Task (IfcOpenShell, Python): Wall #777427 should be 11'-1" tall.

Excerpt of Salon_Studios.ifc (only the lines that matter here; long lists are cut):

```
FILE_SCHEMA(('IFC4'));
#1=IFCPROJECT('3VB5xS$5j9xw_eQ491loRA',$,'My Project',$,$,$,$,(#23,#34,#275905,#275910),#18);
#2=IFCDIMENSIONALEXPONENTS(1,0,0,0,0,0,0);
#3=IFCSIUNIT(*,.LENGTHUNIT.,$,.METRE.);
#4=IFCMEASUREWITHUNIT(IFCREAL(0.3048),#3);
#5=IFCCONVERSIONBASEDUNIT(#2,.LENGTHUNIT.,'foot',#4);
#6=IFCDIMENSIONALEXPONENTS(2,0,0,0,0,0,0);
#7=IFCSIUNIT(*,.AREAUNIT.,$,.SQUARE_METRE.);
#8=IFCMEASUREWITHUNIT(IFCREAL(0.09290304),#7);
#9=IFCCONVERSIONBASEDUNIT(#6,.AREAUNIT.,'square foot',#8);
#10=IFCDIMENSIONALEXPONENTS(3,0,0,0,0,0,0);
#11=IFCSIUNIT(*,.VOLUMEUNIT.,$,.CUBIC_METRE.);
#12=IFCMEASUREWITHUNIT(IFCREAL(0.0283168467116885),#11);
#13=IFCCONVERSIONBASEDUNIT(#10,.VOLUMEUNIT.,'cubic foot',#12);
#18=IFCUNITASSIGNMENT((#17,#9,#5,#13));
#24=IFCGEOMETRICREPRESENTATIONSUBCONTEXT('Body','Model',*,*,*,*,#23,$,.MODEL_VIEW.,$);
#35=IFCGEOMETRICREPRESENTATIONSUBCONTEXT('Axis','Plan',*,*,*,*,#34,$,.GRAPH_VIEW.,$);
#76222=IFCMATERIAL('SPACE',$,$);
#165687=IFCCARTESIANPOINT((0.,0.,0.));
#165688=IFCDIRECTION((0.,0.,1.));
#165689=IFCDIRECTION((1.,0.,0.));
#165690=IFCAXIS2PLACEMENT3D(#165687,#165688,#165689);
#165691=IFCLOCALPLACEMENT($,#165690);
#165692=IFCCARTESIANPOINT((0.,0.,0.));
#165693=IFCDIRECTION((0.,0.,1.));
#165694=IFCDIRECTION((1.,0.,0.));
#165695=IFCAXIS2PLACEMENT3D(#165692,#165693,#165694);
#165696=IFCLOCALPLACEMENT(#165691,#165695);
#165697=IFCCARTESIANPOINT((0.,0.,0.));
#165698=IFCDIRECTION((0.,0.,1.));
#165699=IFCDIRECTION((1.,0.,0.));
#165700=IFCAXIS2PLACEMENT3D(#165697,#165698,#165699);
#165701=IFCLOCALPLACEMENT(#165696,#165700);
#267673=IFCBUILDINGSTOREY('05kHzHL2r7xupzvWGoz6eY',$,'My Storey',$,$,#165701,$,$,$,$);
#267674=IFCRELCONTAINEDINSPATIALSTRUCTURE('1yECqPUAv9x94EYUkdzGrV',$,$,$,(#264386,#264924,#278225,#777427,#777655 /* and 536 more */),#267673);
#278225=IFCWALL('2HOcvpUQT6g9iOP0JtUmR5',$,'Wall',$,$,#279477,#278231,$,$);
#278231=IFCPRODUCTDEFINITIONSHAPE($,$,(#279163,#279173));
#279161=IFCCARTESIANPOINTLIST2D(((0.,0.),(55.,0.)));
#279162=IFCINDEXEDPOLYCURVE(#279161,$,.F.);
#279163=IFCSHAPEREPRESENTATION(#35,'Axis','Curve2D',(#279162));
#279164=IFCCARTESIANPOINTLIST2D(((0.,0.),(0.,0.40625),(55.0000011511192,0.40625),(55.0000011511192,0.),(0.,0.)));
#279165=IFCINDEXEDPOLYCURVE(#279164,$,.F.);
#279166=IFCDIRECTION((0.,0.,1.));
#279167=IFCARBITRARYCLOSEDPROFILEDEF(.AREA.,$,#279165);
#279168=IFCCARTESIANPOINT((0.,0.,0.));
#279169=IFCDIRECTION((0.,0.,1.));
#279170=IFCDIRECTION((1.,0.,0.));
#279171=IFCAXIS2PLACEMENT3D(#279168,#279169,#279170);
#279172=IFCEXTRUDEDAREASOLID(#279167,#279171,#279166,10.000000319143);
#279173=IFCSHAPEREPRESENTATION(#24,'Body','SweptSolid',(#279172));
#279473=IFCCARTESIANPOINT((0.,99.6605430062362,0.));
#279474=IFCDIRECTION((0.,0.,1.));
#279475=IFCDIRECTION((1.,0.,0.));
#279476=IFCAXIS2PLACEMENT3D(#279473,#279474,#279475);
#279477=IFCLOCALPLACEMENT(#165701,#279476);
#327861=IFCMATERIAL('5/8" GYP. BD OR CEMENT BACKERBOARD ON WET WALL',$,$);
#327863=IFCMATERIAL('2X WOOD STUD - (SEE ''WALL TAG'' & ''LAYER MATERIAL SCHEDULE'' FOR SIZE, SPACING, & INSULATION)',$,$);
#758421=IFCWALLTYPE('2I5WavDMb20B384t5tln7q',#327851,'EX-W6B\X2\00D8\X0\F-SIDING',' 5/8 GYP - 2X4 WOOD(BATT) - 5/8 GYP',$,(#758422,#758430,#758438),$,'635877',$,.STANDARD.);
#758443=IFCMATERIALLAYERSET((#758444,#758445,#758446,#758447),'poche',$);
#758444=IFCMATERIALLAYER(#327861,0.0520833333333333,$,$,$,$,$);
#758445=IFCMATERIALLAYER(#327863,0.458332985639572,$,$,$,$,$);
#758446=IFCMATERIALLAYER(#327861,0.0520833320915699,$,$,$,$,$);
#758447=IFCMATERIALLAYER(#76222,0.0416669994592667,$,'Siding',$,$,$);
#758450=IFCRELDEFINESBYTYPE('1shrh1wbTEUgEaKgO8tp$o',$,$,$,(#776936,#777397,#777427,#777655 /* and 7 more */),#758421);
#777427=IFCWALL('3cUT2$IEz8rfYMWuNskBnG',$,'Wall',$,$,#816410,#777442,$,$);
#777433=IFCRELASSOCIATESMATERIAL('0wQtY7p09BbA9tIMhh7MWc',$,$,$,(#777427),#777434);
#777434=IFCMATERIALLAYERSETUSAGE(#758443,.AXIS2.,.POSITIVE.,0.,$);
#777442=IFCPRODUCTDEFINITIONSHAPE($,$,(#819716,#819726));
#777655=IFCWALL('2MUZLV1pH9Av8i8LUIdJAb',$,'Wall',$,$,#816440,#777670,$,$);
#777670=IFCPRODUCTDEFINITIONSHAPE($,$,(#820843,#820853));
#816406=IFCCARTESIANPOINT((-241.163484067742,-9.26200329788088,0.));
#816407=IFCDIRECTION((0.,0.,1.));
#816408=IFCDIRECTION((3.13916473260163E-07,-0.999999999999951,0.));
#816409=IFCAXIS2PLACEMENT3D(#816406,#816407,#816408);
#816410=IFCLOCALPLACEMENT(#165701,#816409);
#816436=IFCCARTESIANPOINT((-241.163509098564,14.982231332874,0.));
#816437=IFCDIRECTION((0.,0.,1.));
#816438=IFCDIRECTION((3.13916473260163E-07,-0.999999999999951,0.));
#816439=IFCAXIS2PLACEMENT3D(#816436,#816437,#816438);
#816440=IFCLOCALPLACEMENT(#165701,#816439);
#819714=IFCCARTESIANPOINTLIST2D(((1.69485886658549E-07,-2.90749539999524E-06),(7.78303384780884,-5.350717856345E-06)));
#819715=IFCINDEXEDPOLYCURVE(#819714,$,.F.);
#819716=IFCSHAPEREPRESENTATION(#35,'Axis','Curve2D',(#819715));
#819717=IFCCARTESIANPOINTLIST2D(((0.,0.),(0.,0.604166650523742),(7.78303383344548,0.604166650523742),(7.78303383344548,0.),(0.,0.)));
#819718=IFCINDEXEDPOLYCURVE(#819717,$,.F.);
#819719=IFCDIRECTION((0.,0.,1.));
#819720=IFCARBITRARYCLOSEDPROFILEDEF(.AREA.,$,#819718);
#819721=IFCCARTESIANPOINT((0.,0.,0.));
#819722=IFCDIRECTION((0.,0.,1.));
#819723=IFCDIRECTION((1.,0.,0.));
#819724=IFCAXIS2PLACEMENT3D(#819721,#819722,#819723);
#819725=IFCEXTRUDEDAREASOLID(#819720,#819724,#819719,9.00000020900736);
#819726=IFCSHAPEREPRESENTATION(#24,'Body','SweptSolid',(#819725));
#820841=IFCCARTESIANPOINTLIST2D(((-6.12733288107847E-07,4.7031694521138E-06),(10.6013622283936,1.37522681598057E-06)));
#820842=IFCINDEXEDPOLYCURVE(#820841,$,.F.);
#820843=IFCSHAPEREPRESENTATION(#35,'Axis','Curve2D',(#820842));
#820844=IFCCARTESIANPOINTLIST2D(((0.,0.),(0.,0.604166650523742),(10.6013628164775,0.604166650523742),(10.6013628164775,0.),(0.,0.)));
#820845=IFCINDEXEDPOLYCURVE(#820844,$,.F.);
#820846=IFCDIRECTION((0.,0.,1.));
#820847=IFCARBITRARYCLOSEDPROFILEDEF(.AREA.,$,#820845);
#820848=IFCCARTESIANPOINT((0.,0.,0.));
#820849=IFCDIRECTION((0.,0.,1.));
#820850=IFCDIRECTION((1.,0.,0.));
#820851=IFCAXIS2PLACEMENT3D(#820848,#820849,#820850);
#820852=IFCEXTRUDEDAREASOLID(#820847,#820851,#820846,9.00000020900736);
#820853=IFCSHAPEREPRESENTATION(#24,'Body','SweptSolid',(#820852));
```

```python
import ifcopenshell
import ifcopenshell.geom
import ifcopenshell.util.representation
import ifcopenshell.util.shape
import ifcopenshell.util.unit

model = ifcopenshell.open("Salon_Studios.ifc")
unit_scale = ifcopenshell.util.unit.calculate_unit_scale(model)
settings = ifcopenshell.geom.settings()


def volume(element):
    """Net volume in cubic metres, openings subtracted."""
    shape = ifcopenshell.geom.create_shape(settings, element)
    return ifcopenshell.util.shape.get_volume(shape.geometry)


wall = model.by_guid("3cUT2$IEz8rfYMWuNskBnG")
before = volume(wall)

body = ifcopenshell.util.representation.get_representation(wall, "Model", "Body")
solid = body.Items[0]
old_height = solid.Depth
solid.Depth = 133 * 0.0254 / unit_scale
after = volume(wall)

print(f"height {old_height:g} -> {solid.Depth:g}, volume {before:.3f} -> {after:.3f} m3")

model.write("Salon_Studios_rev.ifc")
```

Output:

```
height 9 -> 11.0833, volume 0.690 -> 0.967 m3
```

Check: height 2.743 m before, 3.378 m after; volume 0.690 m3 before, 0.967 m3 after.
